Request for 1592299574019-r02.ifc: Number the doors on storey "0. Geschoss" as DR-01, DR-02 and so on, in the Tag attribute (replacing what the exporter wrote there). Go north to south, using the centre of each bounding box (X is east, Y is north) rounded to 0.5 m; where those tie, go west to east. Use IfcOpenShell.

First a look at what the model holds.

```python
import ifcopenshell
import ifcopenshell.util.element
import ifcopenshell.util.placement

model = ifcopenshell.open("1592299574019-r02.ifc")
print(model.schema)
storey = next(s for s in model.by_type("IfcBuildingStorey") if s.Name == "0. Geschoss")
doors = [e for e in ifcopenshell.util.element.get_decomposition(storey) if e.is_a("IfcDoor")]
for e in sorted(doors, key=lambda e: e.id()):
    origin = ifcopenshell.util.placement.get_local_placement(e.ObjectPlacement)[:3, 3]
    print(e.id(), e.Tag, e.Name, origin.round(2) + 0.0, sep=" | ")
```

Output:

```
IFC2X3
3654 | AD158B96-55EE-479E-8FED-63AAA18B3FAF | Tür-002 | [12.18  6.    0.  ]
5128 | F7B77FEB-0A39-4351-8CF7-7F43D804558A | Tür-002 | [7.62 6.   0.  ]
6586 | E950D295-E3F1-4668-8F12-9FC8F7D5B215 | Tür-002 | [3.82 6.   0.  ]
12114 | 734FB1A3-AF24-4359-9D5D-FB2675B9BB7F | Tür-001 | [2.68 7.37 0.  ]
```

```python
import ifcopenshell
import ifcopenshell.geom
import ifcopenshell.util.element
import ifcopenshell.util.shape

model = ifcopenshell.open("1592299574019-r02.ifc")
settings = ifcopenshell.geom.settings()
settings.set("use-world-coords", True)


def centre(element):
    shape = ifcopenshell.geom.create_shape(settings, element)
    return ifcopenshell.util.shape.get_bbox_centroid(shape.geometry)


storey = next(s for s in model.by_type("IfcBuildingStorey") if s.Name == "0. Geschoss")
doors = [e for e in ifcopenshell.util.element.get_decomposition(storey) if e.is_a("IfcDoor")]

# Insertion points can sit at a corner or the storey origin, so sort by the geometry (in metres).
centres = {e: centre(e) for e in doors}
doors.sort(key=lambda e: (-round(centres[e][1] / 0.5), centres[e][0]))

for i, e in enumerate(doors, start=1):
    number = f"DR-{i:02d}"
    e.Tag = number
    print(e.id(), number)

model.write("1592299574019-r02_v2.ifc")
```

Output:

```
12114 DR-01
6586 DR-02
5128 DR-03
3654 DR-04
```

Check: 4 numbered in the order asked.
